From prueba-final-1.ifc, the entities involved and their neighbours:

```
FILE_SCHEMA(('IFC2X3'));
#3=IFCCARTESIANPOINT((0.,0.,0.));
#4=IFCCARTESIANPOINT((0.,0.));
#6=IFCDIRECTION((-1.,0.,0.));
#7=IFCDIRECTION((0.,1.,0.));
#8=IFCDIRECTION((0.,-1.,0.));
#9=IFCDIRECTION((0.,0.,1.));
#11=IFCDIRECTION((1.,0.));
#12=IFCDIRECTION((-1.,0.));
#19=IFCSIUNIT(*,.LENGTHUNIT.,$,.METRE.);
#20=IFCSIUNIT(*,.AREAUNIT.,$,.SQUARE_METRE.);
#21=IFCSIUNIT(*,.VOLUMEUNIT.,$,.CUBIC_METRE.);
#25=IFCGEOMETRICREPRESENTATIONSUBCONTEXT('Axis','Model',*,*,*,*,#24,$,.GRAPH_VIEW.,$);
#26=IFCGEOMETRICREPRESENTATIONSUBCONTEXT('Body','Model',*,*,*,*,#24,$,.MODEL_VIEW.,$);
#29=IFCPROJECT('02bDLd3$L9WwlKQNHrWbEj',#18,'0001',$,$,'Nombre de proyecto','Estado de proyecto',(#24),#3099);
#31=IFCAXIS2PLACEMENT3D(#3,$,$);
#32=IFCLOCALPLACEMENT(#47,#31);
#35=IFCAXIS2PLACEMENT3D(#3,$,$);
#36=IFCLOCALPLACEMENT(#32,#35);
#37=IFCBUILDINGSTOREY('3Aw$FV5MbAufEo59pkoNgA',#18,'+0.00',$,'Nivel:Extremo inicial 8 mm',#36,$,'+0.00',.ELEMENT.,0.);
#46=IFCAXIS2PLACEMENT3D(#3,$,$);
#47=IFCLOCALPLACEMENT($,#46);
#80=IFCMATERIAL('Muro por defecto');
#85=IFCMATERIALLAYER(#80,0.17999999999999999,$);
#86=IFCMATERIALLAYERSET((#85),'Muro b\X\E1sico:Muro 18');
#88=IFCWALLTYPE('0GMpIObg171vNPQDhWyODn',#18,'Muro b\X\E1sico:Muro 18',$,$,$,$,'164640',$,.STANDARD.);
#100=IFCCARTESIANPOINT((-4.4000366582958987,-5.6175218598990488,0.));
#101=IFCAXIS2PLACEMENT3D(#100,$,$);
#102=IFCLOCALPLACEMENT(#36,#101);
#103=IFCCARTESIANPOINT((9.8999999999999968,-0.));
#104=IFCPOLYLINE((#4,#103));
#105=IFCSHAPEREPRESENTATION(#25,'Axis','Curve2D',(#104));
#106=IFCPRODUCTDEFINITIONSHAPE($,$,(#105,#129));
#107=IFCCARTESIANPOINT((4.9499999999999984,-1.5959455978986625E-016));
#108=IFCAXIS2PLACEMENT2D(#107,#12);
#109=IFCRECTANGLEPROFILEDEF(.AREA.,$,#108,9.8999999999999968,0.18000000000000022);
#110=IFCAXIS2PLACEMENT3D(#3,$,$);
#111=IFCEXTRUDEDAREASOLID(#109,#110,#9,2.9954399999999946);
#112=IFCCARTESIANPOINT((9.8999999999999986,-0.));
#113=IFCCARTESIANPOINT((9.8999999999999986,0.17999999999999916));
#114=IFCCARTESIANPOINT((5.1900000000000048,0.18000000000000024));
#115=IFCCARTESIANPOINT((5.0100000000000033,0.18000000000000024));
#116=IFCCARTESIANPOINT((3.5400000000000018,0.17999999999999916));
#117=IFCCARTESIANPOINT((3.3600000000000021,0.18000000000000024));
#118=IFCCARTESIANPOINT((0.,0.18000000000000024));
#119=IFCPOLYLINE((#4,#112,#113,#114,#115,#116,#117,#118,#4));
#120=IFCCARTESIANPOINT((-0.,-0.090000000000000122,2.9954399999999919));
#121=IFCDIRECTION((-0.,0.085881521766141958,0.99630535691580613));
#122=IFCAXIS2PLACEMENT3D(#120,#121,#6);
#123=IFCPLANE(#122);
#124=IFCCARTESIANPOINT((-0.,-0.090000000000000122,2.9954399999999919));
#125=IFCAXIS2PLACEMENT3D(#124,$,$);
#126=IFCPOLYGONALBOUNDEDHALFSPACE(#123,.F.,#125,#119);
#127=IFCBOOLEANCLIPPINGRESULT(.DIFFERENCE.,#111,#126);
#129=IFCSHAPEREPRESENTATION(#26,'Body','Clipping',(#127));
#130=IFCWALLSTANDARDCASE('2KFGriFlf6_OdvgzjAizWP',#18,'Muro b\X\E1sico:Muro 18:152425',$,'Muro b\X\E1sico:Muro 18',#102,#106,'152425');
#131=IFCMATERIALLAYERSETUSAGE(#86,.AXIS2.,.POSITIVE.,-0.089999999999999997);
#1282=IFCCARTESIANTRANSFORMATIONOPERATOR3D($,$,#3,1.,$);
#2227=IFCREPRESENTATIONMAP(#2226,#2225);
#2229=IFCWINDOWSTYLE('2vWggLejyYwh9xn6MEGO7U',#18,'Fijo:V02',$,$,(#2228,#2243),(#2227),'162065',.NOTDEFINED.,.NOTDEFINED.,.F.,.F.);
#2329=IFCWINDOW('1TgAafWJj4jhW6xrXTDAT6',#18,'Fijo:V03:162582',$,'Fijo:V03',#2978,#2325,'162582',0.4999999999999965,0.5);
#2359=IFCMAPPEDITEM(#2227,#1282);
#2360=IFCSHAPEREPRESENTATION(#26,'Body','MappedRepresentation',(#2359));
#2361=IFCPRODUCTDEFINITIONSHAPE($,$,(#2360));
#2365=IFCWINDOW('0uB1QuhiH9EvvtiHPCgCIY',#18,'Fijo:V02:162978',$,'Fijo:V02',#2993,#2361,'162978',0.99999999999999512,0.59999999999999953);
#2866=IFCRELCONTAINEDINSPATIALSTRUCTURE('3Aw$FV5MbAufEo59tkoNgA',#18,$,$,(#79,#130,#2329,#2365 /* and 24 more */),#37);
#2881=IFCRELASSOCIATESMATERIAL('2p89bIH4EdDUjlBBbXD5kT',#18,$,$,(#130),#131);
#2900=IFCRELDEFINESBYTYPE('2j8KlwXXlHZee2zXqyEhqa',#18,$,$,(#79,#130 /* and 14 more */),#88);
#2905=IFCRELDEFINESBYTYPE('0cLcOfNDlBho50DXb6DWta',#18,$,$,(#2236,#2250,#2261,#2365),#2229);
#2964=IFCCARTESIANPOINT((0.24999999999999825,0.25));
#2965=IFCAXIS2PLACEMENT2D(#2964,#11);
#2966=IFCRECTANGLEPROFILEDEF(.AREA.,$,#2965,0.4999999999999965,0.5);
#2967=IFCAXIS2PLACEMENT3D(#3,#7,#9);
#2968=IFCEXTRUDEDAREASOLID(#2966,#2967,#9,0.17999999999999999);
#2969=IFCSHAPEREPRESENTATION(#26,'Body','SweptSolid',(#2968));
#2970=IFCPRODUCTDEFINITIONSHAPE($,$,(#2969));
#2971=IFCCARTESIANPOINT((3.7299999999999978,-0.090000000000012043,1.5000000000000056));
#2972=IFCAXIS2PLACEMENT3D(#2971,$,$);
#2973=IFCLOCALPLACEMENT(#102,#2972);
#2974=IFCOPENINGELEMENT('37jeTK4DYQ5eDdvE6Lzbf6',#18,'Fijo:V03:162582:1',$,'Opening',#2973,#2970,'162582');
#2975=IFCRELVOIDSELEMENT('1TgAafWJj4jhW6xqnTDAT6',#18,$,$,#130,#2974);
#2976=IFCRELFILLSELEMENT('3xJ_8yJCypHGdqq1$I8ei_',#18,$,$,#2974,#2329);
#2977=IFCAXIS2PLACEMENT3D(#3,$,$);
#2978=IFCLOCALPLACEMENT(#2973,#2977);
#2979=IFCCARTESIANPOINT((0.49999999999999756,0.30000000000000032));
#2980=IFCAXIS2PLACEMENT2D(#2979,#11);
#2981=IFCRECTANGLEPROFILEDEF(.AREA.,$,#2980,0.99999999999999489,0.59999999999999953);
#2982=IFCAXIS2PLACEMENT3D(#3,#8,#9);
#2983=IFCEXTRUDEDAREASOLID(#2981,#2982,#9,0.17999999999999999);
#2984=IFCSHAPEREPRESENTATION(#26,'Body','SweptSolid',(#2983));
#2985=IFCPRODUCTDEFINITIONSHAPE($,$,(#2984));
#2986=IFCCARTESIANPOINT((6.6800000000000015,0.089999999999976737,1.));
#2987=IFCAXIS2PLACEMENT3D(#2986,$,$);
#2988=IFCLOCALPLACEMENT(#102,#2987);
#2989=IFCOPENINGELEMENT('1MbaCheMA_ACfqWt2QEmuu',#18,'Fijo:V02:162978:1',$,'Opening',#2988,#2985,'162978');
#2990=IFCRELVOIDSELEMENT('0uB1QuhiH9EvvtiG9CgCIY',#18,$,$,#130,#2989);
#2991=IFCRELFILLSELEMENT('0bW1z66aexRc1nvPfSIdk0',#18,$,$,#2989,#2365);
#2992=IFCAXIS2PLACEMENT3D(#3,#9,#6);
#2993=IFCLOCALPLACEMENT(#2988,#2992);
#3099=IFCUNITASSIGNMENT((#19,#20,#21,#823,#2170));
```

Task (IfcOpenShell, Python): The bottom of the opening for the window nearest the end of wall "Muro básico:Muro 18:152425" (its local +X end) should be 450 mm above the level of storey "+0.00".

```python
import numpy as np
import ifcopenshell
import ifcopenshell.api.geometry
import ifcopenshell.geom
import ifcopenshell.util.element
import ifcopenshell.util.placement
import ifcopenshell.util.shape
import ifcopenshell.util.unit

model = ifcopenshell.open("prueba-final-1.ifc")
unit_scale = ifcopenshell.util.unit.calculate_unit_scale(model)

window = model.by_guid("0uB1QuhiH9EvvtiHPCgCIY")
opening = window.FillsVoids[0].RelatingOpeningElement
storey = ifcopenshell.util.element.get_container(window, ifc_class="IfcBuildingStorey")
level = ifcopenshell.util.placement.get_local_placement(storey.ObjectPlacement)[2, 3]

# The opening's origin need not be at the sill, so measure its lowest point.
shape = ifcopenshell.geom.create_shape(ifcopenshell.geom.settings(), opening)
bottom = ifcopenshell.util.shape.get_shape_bottom_elevation(shape, shape.geometry) / unit_scale
dz = level + 0.45 - bottom

shift = np.array([0.0, 0.0, dz])
# The window is placed relative to its opening, so it follows when the opening moves.
matrix = ifcopenshell.util.placement.get_local_placement(opening.ObjectPlacement)
matrix[:3, 3] += shift
ifcopenshell.api.geometry.edit_object_placement(
    model, product=opening, matrix=matrix, is_si=False, should_transform_children=True
)

print(f"moved by {dz * unit_scale:+.3f} m")

model.write("prueba-final-1_edited.ifc")
```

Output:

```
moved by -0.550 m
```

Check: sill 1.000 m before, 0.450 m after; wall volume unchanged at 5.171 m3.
